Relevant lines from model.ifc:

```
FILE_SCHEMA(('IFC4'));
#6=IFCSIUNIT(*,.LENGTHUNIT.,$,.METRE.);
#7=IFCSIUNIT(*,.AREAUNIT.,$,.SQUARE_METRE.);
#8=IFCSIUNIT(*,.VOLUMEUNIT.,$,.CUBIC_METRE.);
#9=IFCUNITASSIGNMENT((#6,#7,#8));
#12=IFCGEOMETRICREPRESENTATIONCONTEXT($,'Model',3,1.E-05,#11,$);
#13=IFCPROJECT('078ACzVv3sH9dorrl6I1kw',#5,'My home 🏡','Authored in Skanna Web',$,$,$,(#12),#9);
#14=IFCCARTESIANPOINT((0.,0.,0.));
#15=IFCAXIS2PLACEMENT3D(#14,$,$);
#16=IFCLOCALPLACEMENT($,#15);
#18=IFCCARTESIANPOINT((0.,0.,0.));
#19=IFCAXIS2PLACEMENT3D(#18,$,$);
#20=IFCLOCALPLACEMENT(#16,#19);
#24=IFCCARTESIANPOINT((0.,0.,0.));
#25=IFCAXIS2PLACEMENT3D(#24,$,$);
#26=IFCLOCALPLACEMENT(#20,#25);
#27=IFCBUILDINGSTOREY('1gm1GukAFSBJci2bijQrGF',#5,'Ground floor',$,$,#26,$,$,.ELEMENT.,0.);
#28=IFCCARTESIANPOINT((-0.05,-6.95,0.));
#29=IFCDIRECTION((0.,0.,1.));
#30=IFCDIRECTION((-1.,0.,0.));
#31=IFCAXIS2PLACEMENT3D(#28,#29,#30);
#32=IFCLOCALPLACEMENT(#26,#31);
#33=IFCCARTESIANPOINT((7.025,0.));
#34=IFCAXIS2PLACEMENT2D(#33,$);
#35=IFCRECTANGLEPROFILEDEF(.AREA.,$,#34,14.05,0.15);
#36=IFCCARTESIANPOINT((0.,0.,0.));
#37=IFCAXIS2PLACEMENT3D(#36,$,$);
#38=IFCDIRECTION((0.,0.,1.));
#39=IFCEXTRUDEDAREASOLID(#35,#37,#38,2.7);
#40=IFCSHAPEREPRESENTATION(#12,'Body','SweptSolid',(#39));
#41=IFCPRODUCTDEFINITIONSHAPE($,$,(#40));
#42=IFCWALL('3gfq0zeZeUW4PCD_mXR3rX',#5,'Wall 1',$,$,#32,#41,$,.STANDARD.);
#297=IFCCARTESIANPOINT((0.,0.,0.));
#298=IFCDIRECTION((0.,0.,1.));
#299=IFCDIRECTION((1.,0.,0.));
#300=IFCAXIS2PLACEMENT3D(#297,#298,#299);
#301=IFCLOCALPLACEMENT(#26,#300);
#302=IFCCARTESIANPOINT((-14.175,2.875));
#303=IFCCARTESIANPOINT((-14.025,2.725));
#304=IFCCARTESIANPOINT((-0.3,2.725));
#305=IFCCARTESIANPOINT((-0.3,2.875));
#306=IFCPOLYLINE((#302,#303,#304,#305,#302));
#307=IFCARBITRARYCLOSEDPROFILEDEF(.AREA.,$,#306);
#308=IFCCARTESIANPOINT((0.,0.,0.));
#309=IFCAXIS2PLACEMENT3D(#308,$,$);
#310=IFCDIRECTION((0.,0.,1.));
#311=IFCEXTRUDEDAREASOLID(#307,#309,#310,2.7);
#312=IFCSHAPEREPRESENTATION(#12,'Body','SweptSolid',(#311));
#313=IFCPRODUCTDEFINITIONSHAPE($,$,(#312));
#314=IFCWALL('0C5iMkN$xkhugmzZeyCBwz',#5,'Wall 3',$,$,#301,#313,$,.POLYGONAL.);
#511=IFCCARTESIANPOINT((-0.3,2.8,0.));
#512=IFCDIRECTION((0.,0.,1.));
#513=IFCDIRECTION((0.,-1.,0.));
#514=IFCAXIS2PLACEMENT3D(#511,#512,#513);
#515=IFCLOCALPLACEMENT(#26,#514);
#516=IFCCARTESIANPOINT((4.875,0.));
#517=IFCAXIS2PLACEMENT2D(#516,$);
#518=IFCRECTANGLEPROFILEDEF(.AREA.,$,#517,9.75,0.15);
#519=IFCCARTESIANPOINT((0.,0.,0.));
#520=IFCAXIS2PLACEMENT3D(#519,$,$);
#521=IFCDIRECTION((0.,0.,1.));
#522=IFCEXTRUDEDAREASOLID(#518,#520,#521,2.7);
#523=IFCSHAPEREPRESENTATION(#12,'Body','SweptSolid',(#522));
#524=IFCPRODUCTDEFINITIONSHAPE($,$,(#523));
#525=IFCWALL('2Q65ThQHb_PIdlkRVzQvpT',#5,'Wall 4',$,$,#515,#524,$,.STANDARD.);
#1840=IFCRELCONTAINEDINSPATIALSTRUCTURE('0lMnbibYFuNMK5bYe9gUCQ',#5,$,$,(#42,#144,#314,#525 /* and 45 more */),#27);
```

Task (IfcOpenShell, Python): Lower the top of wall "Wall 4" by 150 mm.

```python
import ifcopenshell
import ifcopenshell.geom
import ifcopenshell.util.shape
import ifcopenshell.util.unit

model = ifcopenshell.open("model.ifc")
unit_scale = ifcopenshell.util.unit.calculate_unit_scale(model)
settings = ifcopenshell.geom.settings()


def volume(element):
    """Net volume in cubic metres, openings subtracted."""
    shape = ifcopenshell.geom.create_shape(settings, element)
    return ifcopenshell.util.shape.get_volume(shape.geometry)


wall = model.by_guid("2Q65ThQHb_PIdlkRVzQvpT")
before = volume(wall)

body = next(r for r in wall.Representation.Representations if r.RepresentationIdentifier == "Body")
solid = body.Items[0]
old_height = solid.Depth
solid.Depth -= 0.15 / unit_scale
after = volume(wall)

print(f"height {old_height:g} -> {solid.Depth:g}, volume {before:.3f} -> {after:.3f} m3")

model.write("model_updated.ifc")
```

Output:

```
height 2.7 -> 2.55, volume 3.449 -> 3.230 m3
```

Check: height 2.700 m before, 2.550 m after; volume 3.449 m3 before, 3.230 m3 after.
